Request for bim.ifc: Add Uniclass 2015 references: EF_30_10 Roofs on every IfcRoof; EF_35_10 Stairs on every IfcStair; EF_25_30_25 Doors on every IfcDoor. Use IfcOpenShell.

First a look at what the model holds.

```python
import ifcopenshell

model = ifcopenshell.open("bim.ifc")
print(model.schema)
print("classifications:", [c.Name for c in model.by_type("IfcClassification")])
for ifc_class in ("IfcDoor", "IfcRoof", "IfcStair", "IfcWall", "IfcWindow"):
    print(ifc_class, len(model.by_type(ifc_class)))
```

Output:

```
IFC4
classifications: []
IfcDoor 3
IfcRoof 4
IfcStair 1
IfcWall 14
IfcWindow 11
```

```python
import ifcopenshell
import ifcopenshell.api.classification

model = ifcopenshell.open("bim.ifc")

system = ifcopenshell.api.classification.add_classification(model, classification="Uniclass 2015")

codes = {
    "IfcRoof": ("EF_30_10", "Roofs"),
    "IfcStair": ("EF_35_10", "Stairs"),
    "IfcDoor": ("EF_25_30_25", "Doors"),
}
for ifc_class, (code, name) in codes.items():
    products = model.by_type(ifc_class)
    ifcopenshell.api.classification.add_reference(
        model, products=products, classification=system, identification=code, name=name
    )
    print(code, len(products))

model.write("bim-out.ifc")
```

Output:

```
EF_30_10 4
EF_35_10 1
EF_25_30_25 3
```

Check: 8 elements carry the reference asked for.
